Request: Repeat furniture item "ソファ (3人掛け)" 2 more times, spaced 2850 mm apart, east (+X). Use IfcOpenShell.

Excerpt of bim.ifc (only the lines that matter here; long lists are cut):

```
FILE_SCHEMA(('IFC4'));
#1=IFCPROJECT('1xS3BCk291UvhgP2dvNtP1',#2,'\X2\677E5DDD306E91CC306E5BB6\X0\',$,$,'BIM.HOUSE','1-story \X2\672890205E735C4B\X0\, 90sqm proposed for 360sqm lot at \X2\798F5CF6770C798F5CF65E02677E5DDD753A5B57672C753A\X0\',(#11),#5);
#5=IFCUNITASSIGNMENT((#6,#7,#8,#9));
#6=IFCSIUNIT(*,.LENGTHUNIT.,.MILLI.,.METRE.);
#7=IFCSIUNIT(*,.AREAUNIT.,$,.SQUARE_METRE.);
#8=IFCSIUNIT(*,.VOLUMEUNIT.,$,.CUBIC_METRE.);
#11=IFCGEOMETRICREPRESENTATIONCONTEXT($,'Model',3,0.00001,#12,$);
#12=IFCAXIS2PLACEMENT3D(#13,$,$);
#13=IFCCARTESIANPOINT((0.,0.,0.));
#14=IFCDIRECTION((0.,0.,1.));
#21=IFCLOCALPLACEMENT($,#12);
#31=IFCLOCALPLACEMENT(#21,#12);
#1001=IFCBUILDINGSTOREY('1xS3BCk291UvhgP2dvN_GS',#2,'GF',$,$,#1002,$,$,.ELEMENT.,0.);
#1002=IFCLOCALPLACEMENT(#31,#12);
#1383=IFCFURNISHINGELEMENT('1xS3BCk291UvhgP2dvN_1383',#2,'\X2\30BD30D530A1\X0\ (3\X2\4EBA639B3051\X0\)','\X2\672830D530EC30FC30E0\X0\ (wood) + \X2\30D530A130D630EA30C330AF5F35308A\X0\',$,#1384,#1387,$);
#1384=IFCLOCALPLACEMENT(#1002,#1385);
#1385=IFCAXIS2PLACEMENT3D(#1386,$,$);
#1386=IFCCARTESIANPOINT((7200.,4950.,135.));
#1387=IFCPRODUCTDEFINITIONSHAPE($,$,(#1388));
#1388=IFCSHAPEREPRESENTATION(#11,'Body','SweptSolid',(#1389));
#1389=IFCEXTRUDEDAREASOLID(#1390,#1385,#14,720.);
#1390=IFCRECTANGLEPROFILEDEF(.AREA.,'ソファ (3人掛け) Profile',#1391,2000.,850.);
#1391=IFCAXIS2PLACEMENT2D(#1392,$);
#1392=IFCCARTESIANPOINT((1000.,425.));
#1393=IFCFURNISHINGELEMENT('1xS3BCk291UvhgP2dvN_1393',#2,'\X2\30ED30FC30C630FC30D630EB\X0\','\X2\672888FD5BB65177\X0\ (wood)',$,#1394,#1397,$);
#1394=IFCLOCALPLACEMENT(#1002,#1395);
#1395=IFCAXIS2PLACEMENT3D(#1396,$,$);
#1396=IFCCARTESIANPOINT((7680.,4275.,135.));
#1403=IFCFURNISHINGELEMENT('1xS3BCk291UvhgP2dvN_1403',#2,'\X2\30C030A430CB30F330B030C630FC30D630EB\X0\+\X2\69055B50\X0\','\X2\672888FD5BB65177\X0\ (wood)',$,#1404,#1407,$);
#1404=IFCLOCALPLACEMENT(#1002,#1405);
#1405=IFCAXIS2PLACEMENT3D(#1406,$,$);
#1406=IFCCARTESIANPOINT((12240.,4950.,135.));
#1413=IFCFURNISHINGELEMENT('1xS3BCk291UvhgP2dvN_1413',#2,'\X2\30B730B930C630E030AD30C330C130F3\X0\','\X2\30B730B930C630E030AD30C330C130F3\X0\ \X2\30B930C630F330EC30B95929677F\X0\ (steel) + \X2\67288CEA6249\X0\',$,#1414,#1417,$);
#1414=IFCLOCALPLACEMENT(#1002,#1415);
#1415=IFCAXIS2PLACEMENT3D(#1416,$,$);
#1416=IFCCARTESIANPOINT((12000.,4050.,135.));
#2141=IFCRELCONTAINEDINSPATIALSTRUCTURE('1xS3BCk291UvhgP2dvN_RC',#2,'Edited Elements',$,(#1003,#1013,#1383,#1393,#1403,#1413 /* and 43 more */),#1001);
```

```python
import numpy as np
import ifcopenshell
import ifcopenshell.api.geometry
import ifcopenshell.api.root
import ifcopenshell.util.element
import ifcopenshell.util.placement
import ifcopenshell.util.unit

model = ifcopenshell.open("bim.ifc")
unit_scale = ifcopenshell.util.unit.calculate_unit_scale(model)


def reuse_history(source, copy):
    """copy_class also copies each property set's owner history, people and application; keep the originals."""
    for rel in copy.IsDefinedBy:
        if rel.is_a("IfcRelDefinesByProperties") and (history := rel.RelatingPropertyDefinition.OwnerHistory):
            rel.RelatingPropertyDefinition.OwnerHistory = source.OwnerHistory
            ifcopenshell.util.element.remove_deep2(model, history)


source = model.by_guid("1xS3BCk291UvhgP2dvN_1383")
base = ifcopenshell.util.placement.get_local_placement(source.ObjectPlacement)
step = np.array([1.0, 0.0, 0.0]) * 2.85 / unit_scale

for i in range(1, 3):
    copy = ifcopenshell.api.root.copy_class(model, product=source)
    copy.Representation = ifcopenshell.util.element.copy_deep(
        model, source.Representation, exclude=["IfcGeometricRepresentationContext", "IfcRepresentationMap"]
    )
    reuse_history(source, copy)
    matrix = base.copy()
    matrix[:3, 3] += i * step
    print("added at", matrix[:3, 3].round(3) + 0.0)
    ifcopenshell.api.geometry.edit_object_placement(model, product=copy, matrix=matrix, is_si=False)

model.write("bim_updated.ifc")
```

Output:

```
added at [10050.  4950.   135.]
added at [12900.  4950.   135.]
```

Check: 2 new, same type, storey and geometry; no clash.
